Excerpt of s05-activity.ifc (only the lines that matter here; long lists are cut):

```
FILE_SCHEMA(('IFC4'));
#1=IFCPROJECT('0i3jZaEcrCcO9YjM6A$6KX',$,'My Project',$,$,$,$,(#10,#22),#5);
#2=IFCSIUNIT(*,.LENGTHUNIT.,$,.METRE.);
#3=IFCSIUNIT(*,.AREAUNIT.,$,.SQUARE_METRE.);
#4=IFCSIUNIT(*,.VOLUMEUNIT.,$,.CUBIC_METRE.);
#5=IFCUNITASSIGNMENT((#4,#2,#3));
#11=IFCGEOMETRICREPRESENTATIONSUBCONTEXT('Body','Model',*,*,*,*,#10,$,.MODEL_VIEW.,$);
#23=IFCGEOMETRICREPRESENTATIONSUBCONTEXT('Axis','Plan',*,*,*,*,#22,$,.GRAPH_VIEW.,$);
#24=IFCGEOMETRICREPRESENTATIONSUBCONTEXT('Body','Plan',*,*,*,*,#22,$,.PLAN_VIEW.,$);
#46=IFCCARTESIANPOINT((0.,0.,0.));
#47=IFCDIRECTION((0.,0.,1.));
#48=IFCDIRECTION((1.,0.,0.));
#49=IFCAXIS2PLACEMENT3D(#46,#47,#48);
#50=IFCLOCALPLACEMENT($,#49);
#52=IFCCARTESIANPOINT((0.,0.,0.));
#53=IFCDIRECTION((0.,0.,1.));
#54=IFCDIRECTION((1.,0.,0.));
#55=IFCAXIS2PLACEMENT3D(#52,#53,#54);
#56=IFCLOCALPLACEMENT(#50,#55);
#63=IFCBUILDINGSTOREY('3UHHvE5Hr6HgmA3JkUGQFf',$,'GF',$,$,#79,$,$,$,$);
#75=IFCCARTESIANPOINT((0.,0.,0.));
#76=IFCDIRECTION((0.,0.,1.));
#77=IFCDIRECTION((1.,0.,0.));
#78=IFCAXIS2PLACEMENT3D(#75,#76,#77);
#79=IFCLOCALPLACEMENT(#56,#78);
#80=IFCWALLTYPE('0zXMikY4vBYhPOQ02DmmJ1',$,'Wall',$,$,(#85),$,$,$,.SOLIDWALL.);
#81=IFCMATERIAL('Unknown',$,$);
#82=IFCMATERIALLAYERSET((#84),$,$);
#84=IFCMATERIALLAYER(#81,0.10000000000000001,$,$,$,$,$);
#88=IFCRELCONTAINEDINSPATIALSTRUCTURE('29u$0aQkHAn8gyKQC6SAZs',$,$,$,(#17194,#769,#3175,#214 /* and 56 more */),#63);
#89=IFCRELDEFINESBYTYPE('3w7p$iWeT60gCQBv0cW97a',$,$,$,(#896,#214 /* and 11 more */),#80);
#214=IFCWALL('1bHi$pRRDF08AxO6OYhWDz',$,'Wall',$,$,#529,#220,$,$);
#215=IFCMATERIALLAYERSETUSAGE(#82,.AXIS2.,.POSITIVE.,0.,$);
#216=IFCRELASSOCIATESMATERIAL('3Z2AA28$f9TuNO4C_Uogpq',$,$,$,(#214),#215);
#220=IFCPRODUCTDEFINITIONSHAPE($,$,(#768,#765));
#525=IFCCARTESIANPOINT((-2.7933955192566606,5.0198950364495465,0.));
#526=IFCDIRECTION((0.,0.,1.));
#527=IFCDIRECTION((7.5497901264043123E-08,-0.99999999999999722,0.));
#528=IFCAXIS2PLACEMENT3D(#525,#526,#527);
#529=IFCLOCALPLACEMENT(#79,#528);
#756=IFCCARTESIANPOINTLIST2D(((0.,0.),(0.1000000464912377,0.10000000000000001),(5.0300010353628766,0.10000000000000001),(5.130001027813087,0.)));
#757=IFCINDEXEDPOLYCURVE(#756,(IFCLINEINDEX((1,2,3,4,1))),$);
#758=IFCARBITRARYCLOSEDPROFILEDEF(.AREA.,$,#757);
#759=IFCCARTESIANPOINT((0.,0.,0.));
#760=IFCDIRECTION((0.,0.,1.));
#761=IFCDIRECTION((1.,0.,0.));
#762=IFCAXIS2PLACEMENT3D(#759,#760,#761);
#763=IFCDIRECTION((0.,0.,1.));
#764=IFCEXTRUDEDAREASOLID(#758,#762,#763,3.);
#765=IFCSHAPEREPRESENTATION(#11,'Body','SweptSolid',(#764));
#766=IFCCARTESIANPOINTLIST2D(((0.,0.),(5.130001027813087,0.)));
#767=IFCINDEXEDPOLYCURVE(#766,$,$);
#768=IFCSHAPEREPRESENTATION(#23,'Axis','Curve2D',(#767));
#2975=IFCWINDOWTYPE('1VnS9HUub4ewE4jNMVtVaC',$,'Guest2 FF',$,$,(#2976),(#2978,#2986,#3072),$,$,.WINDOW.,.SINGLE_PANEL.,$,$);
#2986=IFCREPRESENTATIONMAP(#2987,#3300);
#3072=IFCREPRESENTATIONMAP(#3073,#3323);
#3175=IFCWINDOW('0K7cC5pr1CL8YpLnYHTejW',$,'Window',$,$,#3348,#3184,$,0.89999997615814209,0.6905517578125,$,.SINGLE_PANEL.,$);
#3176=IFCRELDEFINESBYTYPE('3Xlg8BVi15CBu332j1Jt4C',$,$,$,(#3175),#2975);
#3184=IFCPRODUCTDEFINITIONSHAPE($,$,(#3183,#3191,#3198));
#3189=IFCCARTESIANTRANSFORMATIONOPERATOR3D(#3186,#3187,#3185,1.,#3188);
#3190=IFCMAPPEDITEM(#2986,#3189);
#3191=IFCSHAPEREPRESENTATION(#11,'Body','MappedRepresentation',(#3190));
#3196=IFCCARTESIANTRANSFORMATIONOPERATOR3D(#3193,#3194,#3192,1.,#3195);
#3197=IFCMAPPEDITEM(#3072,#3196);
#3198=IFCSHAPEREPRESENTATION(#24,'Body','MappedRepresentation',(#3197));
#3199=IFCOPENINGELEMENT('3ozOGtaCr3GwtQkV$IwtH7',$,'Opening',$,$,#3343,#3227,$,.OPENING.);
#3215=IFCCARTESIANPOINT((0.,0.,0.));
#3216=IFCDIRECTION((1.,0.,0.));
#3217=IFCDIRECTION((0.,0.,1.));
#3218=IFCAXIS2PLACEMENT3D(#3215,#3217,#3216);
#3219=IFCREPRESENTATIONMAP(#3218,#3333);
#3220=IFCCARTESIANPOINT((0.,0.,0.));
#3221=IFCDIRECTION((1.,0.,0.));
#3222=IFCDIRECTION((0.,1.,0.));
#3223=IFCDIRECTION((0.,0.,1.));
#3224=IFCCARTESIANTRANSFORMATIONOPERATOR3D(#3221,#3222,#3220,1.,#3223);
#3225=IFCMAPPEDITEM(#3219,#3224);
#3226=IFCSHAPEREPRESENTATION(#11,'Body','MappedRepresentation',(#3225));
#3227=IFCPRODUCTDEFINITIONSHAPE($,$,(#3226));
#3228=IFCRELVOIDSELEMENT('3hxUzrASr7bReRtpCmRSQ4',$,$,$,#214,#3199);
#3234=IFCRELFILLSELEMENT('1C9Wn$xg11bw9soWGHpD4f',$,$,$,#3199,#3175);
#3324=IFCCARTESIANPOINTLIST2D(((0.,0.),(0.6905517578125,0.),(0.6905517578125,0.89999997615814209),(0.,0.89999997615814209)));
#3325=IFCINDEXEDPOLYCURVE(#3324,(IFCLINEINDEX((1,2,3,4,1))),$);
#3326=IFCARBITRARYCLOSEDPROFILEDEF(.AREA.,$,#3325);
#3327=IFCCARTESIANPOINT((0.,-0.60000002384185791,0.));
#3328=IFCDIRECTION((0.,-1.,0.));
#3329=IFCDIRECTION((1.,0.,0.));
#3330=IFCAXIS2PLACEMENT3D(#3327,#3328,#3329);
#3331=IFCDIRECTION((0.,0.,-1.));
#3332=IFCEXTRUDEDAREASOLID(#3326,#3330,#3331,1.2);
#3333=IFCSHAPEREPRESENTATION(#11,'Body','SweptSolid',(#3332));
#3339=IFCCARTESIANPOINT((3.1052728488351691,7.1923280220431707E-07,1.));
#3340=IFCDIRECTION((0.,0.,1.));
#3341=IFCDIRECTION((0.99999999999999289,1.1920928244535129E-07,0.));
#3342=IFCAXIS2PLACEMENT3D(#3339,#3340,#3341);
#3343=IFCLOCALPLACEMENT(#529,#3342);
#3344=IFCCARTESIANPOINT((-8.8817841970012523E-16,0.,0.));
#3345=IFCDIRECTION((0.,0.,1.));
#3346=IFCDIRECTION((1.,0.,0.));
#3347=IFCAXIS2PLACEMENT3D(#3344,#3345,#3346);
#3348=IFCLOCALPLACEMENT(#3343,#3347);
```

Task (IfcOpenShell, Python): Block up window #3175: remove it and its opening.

```python
import ifcopenshell
import ifcopenshell.api.feature
import ifcopenshell.api.root
import ifcopenshell.geom
import ifcopenshell.util.shape

model = ifcopenshell.open("s05-activity.ifc")
settings = ifcopenshell.geom.settings()


def volume(element):
    """Net volume in cubic metres, openings subtracted."""
    shape = ifcopenshell.geom.create_shape(settings, element)
    return ifcopenshell.util.shape.get_volume(shape.geometry)


window = model.by_guid("0K7cC5pr1CL8YpLnYHTejW")
opening = window.FillsVoids[0].RelatingOpeningElement
wall = opening.VoidsElements[0].RelatingBuildingElement
before = volume(wall)

ifcopenshell.api.root.remove_product(model, product=window)
ifcopenshell.api.feature.remove_feature(model, feature=opening)

after = volume(wall)

print(f"wall volume {before:.3f} -> {after:.3f} m3")

model.write("s05-activity-out.ifc")
```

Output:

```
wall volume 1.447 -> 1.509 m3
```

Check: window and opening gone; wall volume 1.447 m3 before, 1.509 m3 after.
